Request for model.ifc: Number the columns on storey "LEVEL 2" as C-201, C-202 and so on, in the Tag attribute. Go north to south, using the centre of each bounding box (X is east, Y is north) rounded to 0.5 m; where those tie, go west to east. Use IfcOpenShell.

First a look at what the model holds.

```python
import ifcopenshell
import ifcopenshell.util.element
import ifcopenshell.util.placement

model = ifcopenshell.open("model.ifc")
print(model.schema)
storey = next(s for s in model.by_type("IfcBuildingStorey") if s.Name == "LEVEL 2")
columns = [e for e in ifcopenshell.util.element.get_decomposition(storey) if e.is_a("IfcColumn")]
for e in sorted(columns, key=lambda e: e.id()):
    origin = ifcopenshell.util.placement.get_local_placement(e.ObjectPlacement)[:3, 3]
    print(e.id(), e.Tag, e.Name, origin.round(2) + 0.0, sep=" | ")
```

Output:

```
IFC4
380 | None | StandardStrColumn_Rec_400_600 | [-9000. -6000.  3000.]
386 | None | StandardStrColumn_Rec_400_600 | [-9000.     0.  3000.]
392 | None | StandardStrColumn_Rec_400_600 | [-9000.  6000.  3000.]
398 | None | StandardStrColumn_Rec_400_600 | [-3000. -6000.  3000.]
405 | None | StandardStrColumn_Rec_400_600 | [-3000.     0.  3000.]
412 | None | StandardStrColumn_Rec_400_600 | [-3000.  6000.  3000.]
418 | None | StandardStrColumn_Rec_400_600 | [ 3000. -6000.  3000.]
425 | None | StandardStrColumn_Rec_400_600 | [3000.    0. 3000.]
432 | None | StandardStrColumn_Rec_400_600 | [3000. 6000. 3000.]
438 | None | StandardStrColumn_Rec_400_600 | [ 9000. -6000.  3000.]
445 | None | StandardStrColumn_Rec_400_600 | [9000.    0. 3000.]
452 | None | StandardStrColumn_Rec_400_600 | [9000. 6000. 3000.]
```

```python
import ifcopenshell
import ifcopenshell.geom
import ifcopenshell.util.element
import ifcopenshell.util.shape

model = ifcopenshell.open("model.ifc")
settings = ifcopenshell.geom.settings()
settings.set("use-world-coords", True)


def centre(element):
    shape = ifcopenshell.geom.create_shape(settings, element)
    return ifcopenshell.util.shape.get_bbox_centroid(shape.geometry)


storey = next(s for s in model.by_type("IfcBuildingStorey") if s.Name == "LEVEL 2")
columns = [e for e in ifcopenshell.util.element.get_decomposition(storey) if e.is_a("IfcColumn")]

# Insertion points can sit at a corner or the storey origin, so sort by the geometry (in metres).
centres = {e: centre(e) for e in columns}
columns.sort(key=lambda e: (-round(centres[e][1] / 0.5), centres[e][0]))

for i, e in enumerate(columns, start=1):
    number = f"C-2{i:02d}"
    e.Tag = number
    print(e.id(), number)

model.write("model_updated.ifc")
```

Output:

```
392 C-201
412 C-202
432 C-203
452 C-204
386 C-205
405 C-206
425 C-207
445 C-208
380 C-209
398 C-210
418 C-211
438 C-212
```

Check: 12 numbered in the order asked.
